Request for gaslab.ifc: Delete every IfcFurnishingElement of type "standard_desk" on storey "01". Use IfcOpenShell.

First a look at what the model holds.

```python
import ifcopenshell
import ifcopenshell.util.element

model = ifcopenshell.open("gaslab.ifc")
print(model.schema)
storey = next(s for s in model.by_type("IfcBuildingStorey") if s.Name == "01")
furniture = [e for e in ifcopenshell.util.element.get_decomposition(storey) if e.is_a("IfcFurnishingElement")]
seen = {}
for e in furniture:
    element_type = ifcopenshell.util.element.get_type(e)
    name = element_type.Name if element_type not in (None, e) else None
    seen[name] = seen.get(name, 0) + 1
for name, count in sorted(seen.items(), key=str):
    print(count, "x", name)
```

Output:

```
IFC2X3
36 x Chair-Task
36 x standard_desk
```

```python
import ifcopenshell
import ifcopenshell.api.root
import ifcopenshell.util.element

model = ifcopenshell.open("gaslab.ifc")

storey = next(s for s in model.by_type("IfcBuildingStorey") if s.Name == "01")
furniture = [e for e in ifcopenshell.util.element.get_decomposition(storey) if e.is_a("IfcFurnishingElement")]
targets = [e for e in furniture if (t := ifcopenshell.util.element.get_type(e)) not in (None, e) and t.Name == "standard_desk"]

for e in targets:
    ifcopenshell.api.root.remove_product(model, product=e)
print(len(targets), "removed")

model.write("gaslab-out.ifc")
```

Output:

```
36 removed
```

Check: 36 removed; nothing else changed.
